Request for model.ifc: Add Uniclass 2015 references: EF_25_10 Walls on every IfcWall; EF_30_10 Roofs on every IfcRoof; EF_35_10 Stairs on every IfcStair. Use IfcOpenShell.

First a look at what the model holds.

```python
import ifcopenshell

model = ifcopenshell.open("model.ifc")
print(model.schema)
print("classifications:", [c.Name for c in model.by_type("IfcClassification")])
for ifc_class in ("IfcDoor", "IfcRoof", "IfcStair", "IfcWall", "IfcWindow"):
    print(ifc_class, len(model.by_type(ifc_class)))
```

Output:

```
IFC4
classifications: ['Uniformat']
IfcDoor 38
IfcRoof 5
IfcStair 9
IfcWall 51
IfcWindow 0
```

```python
import ifcopenshell
import ifcopenshell.api.classification

model = ifcopenshell.open("model.ifc")

system = ifcopenshell.api.classification.add_classification(model, classification="Uniclass 2015")

codes = {
    "IfcWall": ("EF_25_10", "Walls"),
    "IfcRoof": ("EF_30_10", "Roofs"),
    "IfcStair": ("EF_35_10", "Stairs"),
}
for ifc_class, (code, name) in codes.items():
    products = model.by_type(ifc_class)
    ifcopenshell.api.classification.add_reference(
        model, products=products, classification=system, identification=code, name=name
    )
    print(code, len(products))

model.write("model_rev.ifc")
```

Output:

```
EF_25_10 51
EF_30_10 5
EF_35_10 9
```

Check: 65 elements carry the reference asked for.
